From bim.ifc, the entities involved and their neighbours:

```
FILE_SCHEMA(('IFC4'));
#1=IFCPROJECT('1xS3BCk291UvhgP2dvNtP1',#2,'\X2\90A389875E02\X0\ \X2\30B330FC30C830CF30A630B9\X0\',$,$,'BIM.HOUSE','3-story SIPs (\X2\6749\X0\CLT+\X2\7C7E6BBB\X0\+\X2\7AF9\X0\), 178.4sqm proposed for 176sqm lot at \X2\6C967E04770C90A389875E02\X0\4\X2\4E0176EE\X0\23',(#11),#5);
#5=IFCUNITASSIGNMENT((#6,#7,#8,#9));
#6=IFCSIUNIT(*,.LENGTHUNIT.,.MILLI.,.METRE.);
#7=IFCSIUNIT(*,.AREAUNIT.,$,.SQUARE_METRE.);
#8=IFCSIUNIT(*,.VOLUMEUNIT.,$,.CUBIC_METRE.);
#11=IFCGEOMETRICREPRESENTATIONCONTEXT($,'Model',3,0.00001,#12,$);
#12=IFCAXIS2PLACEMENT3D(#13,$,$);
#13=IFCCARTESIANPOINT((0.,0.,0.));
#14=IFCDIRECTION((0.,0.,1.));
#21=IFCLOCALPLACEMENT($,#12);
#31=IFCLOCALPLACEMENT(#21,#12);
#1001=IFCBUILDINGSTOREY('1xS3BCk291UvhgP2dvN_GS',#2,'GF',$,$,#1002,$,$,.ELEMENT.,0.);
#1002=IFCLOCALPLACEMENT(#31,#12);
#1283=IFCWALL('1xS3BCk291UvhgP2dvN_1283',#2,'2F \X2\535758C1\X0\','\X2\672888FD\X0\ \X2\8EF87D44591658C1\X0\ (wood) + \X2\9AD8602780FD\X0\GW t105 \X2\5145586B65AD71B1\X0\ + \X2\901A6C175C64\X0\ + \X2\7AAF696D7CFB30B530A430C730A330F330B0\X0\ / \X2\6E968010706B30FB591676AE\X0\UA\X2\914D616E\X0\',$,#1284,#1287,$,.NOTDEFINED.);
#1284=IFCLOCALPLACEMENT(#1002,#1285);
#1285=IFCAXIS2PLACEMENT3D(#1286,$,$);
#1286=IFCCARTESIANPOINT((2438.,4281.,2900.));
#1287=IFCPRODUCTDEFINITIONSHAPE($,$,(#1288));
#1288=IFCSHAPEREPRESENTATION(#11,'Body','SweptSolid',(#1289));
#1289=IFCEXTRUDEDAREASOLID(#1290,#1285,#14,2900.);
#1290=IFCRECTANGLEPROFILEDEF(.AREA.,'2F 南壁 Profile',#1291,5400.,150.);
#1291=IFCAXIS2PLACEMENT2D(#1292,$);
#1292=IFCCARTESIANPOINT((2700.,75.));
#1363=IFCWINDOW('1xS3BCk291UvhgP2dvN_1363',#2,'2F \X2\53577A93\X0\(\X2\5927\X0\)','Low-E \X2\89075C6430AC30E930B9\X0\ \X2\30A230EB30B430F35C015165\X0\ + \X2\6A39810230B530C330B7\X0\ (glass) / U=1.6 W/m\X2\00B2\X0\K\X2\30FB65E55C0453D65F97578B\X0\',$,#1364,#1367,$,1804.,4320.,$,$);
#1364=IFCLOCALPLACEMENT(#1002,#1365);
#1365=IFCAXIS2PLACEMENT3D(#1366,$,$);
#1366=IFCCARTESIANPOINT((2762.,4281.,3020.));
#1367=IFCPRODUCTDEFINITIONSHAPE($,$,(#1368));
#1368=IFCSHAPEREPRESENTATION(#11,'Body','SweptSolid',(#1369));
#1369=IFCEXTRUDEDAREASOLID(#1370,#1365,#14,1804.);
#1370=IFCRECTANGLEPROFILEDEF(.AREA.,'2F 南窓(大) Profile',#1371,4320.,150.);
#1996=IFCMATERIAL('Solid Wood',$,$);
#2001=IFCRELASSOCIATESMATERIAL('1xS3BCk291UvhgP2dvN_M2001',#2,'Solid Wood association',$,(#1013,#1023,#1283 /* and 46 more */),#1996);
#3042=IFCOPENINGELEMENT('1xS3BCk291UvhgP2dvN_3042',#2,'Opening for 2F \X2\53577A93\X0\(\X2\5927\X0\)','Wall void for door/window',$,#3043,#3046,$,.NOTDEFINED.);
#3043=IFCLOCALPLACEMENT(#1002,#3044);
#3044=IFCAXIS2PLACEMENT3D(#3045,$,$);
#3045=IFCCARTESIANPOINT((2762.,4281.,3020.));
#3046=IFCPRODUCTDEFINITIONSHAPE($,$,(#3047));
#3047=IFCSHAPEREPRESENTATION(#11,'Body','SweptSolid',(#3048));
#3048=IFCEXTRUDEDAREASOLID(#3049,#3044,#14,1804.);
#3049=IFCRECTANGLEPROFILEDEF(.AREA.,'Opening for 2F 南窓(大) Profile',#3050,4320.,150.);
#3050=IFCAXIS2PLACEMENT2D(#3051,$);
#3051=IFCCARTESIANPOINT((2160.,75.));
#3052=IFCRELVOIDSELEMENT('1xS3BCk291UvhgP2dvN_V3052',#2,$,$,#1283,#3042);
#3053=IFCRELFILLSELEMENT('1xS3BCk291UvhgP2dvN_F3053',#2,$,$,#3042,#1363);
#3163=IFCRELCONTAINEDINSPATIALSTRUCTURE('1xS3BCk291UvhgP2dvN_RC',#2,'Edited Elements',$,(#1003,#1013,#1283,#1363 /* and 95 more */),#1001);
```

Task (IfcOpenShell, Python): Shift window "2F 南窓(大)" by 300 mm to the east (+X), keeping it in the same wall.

```python
import ifcopenshell
import ifcopenshell.api.geometry
import ifcopenshell.util.placement

model = ifcopenshell.open("bim.ifc")

window = model.by_id(1363)
opening = window.FillsVoids[0].RelatingOpeningElement
wall = opening.VoidsElements[0].RelatingBuildingElement

wall_matrix = ifcopenshell.util.placement.get_local_placement(wall.ObjectPlacement)
shift = wall_matrix[:3, 0] * 300.0
before = ifcopenshell.util.placement.get_local_placement(window.ObjectPlacement)[:3, 3].copy()

# The window is not placed relative to its opening, so move both.
for product in (opening, window):
    matrix = ifcopenshell.util.placement.get_local_placement(product.ObjectPlacement)
    matrix[:3, 3] += shift
    ifcopenshell.api.geometry.edit_object_placement(model, product=product, matrix=matrix, is_si=False)

after = ifcopenshell.util.placement.get_local_placement(window.ObjectPlacement)[:3, 3]
print("window moved by", (after - before).round(3) + 0.0)

model.write("bim_rev.ifc")
```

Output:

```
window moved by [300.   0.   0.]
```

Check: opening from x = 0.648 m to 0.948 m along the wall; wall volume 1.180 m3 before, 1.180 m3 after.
